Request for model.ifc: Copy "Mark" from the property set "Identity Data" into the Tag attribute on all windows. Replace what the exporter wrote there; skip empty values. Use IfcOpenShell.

First a look at what the model holds.

```python
import ifcopenshell
import ifcopenshell.util.element

model = ifcopenshell.open("model.ifc")
print(model.schema)
windows = model.by_type("IfcWindow")
print(len(windows), "windows")
for e in windows[:8]:
    source = ifcopenshell.util.element.get_pset(e, "Identity Data", "Mark")
    target = e.Tag
    print(e.id(), repr(source), repr(target), sep=" | ")
```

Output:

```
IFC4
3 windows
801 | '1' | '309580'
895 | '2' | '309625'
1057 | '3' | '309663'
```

```python
import ifcopenshell
import ifcopenshell.util.element

model = ifcopenshell.open("model.ifc")

count = 0
for e in model.by_type("IfcWindow"):
    value = ifcopenshell.util.element.get_pset(e, "Identity Data", "Mark")
    current = e.Tag
    if not value or not value.strip() or current == value:
        continue
    e.Tag = value
    count += 1

print(count, "windows updated")

model.write("model_v2.ifc")
```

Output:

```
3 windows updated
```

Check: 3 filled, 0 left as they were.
